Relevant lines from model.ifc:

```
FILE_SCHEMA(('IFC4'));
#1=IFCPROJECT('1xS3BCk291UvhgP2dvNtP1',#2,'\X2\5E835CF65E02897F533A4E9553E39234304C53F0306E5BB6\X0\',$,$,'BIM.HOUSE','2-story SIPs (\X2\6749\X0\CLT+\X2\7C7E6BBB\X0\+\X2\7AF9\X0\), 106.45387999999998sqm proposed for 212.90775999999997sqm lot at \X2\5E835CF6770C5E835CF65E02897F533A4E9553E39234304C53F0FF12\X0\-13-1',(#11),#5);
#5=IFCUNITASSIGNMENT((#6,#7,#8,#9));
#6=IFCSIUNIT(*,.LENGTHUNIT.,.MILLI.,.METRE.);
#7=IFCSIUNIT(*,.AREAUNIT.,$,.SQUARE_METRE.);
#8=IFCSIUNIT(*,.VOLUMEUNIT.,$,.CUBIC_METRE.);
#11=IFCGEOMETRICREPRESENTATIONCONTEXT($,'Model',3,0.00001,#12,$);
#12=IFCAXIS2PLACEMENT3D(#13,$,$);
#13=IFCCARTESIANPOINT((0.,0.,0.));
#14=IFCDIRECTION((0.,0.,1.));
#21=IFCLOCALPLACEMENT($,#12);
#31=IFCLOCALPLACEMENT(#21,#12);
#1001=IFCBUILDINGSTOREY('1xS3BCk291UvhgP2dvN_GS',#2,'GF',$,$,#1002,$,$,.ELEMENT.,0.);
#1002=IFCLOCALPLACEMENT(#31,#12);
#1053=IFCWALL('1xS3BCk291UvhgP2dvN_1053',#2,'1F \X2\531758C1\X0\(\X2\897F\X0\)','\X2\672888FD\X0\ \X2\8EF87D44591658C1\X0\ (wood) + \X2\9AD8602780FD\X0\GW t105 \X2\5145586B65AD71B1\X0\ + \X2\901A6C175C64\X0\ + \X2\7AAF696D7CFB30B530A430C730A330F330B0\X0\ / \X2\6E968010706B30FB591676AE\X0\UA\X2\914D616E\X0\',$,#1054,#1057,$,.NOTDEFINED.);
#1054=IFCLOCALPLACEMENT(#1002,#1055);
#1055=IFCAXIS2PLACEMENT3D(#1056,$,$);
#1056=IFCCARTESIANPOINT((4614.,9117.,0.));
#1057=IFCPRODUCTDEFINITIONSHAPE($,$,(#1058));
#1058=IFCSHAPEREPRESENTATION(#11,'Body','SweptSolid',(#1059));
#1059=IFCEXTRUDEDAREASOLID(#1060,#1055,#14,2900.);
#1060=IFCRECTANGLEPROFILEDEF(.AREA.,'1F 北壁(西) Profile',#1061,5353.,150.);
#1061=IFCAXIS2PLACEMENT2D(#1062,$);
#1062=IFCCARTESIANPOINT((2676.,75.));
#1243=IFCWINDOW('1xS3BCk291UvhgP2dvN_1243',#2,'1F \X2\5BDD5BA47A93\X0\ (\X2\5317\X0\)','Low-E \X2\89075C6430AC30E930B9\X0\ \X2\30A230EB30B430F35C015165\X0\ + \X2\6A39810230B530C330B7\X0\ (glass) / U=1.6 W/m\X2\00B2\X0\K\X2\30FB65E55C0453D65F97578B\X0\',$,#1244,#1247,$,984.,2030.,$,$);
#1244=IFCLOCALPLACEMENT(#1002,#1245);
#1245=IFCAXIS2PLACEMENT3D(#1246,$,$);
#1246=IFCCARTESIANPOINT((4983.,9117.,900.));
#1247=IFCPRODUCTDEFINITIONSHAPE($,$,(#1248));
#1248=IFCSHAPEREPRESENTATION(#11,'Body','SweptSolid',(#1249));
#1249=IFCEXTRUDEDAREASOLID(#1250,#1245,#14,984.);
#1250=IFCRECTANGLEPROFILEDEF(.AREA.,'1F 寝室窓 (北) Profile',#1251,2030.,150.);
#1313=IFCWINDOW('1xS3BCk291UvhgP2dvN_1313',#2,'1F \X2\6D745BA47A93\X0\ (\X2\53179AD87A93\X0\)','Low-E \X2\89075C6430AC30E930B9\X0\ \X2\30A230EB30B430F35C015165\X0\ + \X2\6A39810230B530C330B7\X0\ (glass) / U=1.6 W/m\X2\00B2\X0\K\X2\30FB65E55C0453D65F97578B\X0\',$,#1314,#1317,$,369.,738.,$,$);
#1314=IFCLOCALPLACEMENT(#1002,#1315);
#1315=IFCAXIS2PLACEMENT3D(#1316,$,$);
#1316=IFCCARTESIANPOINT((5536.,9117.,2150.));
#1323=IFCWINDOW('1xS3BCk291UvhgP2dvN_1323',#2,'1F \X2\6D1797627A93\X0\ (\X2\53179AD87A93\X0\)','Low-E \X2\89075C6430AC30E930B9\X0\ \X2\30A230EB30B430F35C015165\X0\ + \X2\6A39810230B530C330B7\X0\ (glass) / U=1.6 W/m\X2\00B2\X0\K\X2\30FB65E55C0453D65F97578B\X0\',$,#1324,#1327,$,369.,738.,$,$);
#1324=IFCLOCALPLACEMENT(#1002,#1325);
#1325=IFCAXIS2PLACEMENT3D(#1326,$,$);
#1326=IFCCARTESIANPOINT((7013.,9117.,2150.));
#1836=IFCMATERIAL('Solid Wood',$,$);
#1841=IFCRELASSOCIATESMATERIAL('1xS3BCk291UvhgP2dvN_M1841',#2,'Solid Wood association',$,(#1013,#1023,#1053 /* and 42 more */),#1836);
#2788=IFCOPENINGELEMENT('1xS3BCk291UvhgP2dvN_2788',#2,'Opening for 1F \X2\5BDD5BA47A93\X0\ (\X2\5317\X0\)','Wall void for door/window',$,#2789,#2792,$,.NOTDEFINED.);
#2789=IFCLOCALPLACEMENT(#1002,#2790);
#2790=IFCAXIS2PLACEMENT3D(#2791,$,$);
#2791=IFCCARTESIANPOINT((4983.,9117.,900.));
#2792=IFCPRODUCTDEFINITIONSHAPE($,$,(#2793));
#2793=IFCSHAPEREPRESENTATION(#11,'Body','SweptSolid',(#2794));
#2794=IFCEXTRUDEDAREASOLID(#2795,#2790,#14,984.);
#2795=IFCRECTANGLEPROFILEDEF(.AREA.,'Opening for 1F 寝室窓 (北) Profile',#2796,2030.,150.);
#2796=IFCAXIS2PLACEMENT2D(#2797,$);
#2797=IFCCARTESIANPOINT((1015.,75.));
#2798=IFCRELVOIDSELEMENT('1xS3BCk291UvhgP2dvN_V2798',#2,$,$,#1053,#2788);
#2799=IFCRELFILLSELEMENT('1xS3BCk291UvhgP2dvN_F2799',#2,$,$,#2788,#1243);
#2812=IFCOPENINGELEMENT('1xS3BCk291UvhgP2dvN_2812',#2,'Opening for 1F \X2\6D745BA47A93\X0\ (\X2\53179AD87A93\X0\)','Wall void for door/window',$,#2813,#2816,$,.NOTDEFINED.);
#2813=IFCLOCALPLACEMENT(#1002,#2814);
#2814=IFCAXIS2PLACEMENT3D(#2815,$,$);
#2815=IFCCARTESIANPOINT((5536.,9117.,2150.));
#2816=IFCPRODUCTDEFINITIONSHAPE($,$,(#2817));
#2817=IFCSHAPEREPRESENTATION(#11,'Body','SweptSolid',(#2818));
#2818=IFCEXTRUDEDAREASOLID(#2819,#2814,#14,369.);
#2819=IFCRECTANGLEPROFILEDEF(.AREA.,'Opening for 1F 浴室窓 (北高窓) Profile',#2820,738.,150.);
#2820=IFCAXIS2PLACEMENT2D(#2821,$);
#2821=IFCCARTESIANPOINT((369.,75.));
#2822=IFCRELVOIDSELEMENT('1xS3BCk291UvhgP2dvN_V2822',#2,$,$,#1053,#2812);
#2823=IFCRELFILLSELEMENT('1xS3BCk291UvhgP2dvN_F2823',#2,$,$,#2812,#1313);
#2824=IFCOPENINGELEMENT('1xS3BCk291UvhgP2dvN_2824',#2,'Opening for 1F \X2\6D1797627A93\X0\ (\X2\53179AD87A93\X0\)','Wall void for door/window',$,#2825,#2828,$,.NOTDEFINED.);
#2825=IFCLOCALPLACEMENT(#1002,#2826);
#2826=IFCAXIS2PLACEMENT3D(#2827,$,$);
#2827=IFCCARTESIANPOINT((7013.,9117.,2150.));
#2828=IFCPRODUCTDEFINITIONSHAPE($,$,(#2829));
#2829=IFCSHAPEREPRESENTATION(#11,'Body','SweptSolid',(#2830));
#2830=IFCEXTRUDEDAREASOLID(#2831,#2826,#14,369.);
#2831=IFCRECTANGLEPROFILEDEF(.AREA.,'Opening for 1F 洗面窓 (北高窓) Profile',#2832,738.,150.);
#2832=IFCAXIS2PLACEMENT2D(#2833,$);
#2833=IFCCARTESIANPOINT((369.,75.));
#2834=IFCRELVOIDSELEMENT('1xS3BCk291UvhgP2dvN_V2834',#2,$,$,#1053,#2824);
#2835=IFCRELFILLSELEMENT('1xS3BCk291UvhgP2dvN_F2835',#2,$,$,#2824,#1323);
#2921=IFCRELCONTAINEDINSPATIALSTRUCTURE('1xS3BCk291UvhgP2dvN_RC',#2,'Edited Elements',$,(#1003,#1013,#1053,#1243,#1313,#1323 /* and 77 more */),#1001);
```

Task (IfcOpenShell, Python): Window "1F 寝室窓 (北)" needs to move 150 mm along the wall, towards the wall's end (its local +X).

```python
import ifcopenshell
import ifcopenshell.api.geometry
import ifcopenshell.util.placement
import ifcopenshell.util.unit

model = ifcopenshell.open("model.ifc")
unit_scale = ifcopenshell.util.unit.calculate_unit_scale(model)

window = model.by_guid("1xS3BCk291UvhgP2dvN_1243")
opening = window.FillsVoids[0].RelatingOpeningElement
wall = opening.VoidsElements[0].RelatingBuildingElement

wall_matrix = ifcopenshell.util.placement.get_local_placement(wall.ObjectPlacement)
shift = wall_matrix[:3, 0] * 0.15 / unit_scale
before = ifcopenshell.util.placement.get_local_placement(window.ObjectPlacement)[:3, 3].copy()

# The window is not placed relative to its opening, so move both.
for product in (opening, window):
    matrix = ifcopenshell.util.placement.get_local_placement(product.ObjectPlacement)
    matrix[:3, 3] += shift
    ifcopenshell.api.geometry.edit_object_placement(model, product=product, matrix=matrix, is_si=False)

after = ifcopenshell.util.placement.get_local_placement(window.ObjectPlacement)[:3, 3]
print("window moved by", (after - before).round(3) + 0.0)

model.write("model-out.ifc")
```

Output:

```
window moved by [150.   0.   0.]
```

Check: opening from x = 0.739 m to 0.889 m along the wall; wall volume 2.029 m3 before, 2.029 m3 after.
